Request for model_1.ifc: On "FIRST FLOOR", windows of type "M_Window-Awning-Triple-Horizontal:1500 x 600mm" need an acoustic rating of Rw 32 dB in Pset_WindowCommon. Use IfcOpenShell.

First a look at what the model holds.

```python
import ifcopenshell
import ifcopenshell.util.element

model = ifcopenshell.open("model_1.ifc")
print(model.schema)
storey = next(s for s in model.by_type("IfcBuildingStorey") if s.Name == "FIRST FLOOR")
windows = [e for e in ifcopenshell.util.element.get_decomposition(storey) if e.is_a("IfcWindow")]
seen = {}
for e in windows:
    element_type = ifcopenshell.util.element.get_type(e)
    key = (element_type.Name if element_type != e and element_type else None, ifcopenshell.util.element.get_pset(e, "Pset_WindowCommon", "AcousticRating"))
    seen[key] = seen.get(key, 0) + 1
for (name, value), count in sorted(seen.items(), key=str):
    print(count, "x", name, "|", value)
```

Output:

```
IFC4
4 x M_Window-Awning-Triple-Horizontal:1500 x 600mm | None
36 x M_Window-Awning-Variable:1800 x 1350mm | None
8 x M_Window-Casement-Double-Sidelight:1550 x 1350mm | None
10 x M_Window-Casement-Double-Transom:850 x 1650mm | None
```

```python
import ifcopenshell
import ifcopenshell.api.pset
import ifcopenshell.util.element

model = ifcopenshell.open("model_1.ifc")

storey = next(s for s in model.by_type("IfcBuildingStorey") if s.Name == "FIRST FLOOR")
windows = [e for e in ifcopenshell.util.element.get_decomposition(storey) if e.is_a("IfcWindow")]

count = 0
for e in windows:
    element_type = ifcopenshell.util.element.get_type(e)
    if element_type in (None, e) or element_type.Name != "M_Window-Awning-Triple-Horizontal:1500 x 600mm":
        continue
    # add_pset returns the element's existing set when there is one.
    pset = ifcopenshell.api.pset.add_pset(model, product=e, name="Pset_WindowCommon")
    ifcopenshell.api.pset.edit_pset(model, pset=pset, properties={"AcousticRating": "Rw 32 dB"})
    count += 1

print(count, "windows updated")

model.write("model_1_rev.ifc")
```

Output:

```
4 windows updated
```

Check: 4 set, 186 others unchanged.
